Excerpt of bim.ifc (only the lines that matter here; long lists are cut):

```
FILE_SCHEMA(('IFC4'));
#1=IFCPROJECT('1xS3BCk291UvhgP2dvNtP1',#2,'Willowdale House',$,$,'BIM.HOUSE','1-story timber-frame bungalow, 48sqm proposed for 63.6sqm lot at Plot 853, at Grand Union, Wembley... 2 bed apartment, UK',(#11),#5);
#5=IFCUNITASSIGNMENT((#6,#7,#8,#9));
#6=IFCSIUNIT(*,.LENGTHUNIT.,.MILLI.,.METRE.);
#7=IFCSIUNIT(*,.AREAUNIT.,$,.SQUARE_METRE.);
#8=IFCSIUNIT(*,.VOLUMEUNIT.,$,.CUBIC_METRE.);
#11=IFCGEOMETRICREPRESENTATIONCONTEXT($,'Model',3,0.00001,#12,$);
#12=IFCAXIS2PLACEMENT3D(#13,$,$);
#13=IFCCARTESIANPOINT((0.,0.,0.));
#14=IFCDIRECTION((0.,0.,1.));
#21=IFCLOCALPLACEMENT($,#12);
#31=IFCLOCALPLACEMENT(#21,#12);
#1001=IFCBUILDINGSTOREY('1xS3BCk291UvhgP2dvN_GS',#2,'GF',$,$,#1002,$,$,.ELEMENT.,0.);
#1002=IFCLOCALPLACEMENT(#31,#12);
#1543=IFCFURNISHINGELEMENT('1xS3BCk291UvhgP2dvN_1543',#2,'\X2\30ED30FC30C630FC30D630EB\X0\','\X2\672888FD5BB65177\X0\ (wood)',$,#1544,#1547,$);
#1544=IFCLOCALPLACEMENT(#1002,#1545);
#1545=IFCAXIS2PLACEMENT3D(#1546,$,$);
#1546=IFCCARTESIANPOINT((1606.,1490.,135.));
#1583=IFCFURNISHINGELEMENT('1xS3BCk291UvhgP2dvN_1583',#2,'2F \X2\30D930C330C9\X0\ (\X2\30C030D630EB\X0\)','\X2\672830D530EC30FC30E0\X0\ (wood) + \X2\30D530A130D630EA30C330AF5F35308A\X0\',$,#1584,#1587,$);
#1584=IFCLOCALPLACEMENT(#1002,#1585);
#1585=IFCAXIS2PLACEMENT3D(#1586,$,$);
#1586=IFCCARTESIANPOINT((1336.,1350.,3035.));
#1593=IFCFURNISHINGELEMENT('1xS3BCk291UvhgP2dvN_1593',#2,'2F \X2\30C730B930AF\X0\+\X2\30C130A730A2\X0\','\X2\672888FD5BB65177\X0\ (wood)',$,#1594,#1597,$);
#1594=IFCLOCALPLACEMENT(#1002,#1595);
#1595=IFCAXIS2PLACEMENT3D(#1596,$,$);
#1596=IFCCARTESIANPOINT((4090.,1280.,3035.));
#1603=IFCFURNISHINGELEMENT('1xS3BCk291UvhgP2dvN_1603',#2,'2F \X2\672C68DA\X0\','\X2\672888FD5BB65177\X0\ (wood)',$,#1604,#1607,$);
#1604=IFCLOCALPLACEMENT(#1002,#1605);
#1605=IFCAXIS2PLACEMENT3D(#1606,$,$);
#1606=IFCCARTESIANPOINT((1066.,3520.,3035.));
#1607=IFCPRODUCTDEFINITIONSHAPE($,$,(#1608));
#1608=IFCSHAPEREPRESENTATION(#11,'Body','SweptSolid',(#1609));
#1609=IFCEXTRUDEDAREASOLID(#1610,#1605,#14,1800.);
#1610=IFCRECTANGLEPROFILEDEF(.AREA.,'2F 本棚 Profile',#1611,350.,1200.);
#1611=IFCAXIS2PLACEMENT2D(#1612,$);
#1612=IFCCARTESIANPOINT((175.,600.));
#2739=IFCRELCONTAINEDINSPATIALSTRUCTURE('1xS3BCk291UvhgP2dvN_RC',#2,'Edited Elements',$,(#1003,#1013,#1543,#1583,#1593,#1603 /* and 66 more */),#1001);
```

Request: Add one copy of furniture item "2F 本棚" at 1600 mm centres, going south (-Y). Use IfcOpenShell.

```python
import numpy as np
import ifcopenshell
import ifcopenshell.api.geometry
import ifcopenshell.api.root
import ifcopenshell.util.element
import ifcopenshell.util.placement
import ifcopenshell.util.unit

model = ifcopenshell.open("bim.ifc")
unit_scale = ifcopenshell.util.unit.calculate_unit_scale(model)


def reuse_history(source, copy):
    """copy_class also copies each property set's owner history, people and application; keep the originals."""
    for rel in copy.IsDefinedBy:
        if rel.is_a("IfcRelDefinesByProperties") and (history := rel.RelatingPropertyDefinition.OwnerHistory):
            rel.RelatingPropertyDefinition.OwnerHistory = source.OwnerHistory
            ifcopenshell.util.element.remove_deep2(model, history)


source = model.by_id(1603)
base = ifcopenshell.util.placement.get_local_placement(source.ObjectPlacement)
step = np.array([0.0, -1.0, 0.0]) * 1.6 / unit_scale

for i in range(1, 2):
    copy = ifcopenshell.api.root.copy_class(model, product=source)
    copy.Representation = ifcopenshell.util.element.copy_deep(
        model, source.Representation, exclude=["IfcGeometricRepresentationContext", "IfcRepresentationMap"]
    )
    reuse_history(source, copy)
    matrix = base.copy()
    matrix[:3, 3] += i * step
    print("added at", matrix[:3, 3].round(3) + 0.0)
    ifcopenshell.api.geometry.edit_object_placement(model, product=copy, matrix=matrix, is_si=False)

model.write("bim_edited.ifc")
```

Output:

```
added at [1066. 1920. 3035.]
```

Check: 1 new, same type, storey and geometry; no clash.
